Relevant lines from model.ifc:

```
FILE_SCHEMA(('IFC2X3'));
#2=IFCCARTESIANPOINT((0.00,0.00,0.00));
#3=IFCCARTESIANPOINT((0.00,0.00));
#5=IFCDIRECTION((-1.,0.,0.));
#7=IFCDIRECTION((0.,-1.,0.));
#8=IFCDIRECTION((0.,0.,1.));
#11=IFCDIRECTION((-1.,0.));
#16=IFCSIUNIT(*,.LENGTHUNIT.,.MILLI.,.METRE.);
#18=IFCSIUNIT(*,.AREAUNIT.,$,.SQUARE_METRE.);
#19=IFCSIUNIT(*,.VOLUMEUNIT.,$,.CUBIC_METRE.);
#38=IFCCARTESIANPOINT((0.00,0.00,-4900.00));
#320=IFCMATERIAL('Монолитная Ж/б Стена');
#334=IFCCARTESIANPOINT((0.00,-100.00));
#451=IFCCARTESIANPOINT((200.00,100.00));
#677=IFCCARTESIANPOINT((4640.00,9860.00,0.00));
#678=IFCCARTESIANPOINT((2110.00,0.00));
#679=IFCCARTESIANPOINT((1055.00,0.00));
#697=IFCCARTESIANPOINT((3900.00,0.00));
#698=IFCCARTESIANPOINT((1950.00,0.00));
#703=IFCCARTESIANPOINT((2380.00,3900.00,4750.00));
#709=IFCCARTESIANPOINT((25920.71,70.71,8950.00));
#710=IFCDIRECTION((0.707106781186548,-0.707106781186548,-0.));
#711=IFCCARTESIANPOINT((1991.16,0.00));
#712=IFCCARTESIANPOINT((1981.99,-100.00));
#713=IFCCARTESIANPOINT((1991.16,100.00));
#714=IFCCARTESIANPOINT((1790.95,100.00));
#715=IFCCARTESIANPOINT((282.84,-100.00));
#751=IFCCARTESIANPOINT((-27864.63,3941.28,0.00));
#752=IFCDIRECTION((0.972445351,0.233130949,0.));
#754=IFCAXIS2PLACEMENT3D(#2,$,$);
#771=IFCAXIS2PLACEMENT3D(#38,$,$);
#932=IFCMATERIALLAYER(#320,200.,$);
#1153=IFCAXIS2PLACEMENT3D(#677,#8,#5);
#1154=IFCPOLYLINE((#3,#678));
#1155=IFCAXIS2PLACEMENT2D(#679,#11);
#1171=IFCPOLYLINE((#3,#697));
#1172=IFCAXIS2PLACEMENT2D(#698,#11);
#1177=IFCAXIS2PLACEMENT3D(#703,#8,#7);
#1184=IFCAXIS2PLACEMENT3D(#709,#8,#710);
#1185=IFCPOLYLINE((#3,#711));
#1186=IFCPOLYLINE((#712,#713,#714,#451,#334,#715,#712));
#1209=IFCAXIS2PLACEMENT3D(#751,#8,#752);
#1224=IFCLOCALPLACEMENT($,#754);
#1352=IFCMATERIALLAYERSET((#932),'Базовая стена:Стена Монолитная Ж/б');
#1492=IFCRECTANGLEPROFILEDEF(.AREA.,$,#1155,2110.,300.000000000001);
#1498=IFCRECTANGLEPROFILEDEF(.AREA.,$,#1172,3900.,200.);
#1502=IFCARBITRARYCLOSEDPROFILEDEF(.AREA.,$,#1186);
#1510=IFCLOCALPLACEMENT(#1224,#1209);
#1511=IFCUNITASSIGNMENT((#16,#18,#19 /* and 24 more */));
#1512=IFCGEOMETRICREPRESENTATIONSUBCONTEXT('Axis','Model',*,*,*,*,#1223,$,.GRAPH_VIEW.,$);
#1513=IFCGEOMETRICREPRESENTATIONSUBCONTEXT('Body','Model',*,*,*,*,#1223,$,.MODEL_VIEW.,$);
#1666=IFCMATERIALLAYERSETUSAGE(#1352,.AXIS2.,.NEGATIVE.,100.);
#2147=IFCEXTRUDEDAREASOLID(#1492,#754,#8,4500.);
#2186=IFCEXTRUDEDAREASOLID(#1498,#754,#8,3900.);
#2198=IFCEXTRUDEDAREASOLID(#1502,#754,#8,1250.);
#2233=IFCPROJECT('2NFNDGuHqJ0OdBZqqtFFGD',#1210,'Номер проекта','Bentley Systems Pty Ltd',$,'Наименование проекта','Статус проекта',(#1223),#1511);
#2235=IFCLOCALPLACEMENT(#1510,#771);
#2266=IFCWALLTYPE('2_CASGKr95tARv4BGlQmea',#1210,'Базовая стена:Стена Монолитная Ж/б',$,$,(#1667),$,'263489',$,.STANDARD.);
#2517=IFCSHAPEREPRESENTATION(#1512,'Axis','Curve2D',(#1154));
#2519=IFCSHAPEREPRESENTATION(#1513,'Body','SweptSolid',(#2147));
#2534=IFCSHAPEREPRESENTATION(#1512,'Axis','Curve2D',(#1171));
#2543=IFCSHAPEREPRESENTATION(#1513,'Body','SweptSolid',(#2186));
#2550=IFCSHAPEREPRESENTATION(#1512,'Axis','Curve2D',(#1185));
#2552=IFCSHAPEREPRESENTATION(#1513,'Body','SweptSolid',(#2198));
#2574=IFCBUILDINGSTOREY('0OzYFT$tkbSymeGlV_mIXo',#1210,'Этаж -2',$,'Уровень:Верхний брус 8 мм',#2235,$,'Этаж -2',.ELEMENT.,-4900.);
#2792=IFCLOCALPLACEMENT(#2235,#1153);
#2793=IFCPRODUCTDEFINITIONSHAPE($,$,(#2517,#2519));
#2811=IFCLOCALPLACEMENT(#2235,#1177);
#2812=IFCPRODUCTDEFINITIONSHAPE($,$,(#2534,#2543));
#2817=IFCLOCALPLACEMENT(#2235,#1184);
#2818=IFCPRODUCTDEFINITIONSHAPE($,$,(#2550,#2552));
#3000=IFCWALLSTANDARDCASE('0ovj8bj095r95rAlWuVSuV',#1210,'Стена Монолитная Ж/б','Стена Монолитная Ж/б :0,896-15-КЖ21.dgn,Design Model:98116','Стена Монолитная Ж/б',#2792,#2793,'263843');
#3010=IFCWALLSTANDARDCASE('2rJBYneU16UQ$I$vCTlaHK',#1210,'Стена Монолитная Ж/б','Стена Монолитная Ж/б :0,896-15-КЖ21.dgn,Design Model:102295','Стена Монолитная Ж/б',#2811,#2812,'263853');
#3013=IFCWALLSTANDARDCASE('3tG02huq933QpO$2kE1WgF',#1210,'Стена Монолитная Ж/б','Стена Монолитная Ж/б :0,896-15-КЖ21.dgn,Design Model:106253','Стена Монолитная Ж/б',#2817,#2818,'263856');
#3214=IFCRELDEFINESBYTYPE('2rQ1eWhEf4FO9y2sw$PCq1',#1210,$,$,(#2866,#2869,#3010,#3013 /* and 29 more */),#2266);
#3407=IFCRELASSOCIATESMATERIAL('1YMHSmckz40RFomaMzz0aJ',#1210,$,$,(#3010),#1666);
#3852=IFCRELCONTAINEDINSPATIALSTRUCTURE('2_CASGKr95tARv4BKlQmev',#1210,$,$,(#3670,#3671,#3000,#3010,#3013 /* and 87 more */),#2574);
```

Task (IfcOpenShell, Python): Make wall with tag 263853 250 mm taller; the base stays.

```python
import ifcopenshell
import ifcopenshell.geom
import ifcopenshell.util.representation
import ifcopenshell.util.shape
import ifcopenshell.util.unit

model = ifcopenshell.open("model.ifc")
unit_scale = ifcopenshell.util.unit.calculate_unit_scale(model)
settings = ifcopenshell.geom.settings()


def volume(element):
    """Net volume in cubic metres, openings subtracted."""
    shape = ifcopenshell.geom.create_shape(settings, element)
    return ifcopenshell.util.shape.get_volume(shape.geometry)


wall = model.by_guid("2rJBYneU16UQ$I$vCTlaHK")
before = volume(wall)

body = ifcopenshell.util.representation.get_representation(wall, "Model", "Body")
solid = body.Items[0]
old_height = solid.Depth
solid.Depth += 0.25 / unit_scale
after = volume(wall)

print(f"height {old_height:g} -> {solid.Depth:g}, volume {before:.3f} -> {after:.3f} m3")

model.write("model_edited.ifc")
```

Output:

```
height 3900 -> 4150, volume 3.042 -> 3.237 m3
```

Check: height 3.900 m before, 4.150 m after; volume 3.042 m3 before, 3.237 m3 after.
